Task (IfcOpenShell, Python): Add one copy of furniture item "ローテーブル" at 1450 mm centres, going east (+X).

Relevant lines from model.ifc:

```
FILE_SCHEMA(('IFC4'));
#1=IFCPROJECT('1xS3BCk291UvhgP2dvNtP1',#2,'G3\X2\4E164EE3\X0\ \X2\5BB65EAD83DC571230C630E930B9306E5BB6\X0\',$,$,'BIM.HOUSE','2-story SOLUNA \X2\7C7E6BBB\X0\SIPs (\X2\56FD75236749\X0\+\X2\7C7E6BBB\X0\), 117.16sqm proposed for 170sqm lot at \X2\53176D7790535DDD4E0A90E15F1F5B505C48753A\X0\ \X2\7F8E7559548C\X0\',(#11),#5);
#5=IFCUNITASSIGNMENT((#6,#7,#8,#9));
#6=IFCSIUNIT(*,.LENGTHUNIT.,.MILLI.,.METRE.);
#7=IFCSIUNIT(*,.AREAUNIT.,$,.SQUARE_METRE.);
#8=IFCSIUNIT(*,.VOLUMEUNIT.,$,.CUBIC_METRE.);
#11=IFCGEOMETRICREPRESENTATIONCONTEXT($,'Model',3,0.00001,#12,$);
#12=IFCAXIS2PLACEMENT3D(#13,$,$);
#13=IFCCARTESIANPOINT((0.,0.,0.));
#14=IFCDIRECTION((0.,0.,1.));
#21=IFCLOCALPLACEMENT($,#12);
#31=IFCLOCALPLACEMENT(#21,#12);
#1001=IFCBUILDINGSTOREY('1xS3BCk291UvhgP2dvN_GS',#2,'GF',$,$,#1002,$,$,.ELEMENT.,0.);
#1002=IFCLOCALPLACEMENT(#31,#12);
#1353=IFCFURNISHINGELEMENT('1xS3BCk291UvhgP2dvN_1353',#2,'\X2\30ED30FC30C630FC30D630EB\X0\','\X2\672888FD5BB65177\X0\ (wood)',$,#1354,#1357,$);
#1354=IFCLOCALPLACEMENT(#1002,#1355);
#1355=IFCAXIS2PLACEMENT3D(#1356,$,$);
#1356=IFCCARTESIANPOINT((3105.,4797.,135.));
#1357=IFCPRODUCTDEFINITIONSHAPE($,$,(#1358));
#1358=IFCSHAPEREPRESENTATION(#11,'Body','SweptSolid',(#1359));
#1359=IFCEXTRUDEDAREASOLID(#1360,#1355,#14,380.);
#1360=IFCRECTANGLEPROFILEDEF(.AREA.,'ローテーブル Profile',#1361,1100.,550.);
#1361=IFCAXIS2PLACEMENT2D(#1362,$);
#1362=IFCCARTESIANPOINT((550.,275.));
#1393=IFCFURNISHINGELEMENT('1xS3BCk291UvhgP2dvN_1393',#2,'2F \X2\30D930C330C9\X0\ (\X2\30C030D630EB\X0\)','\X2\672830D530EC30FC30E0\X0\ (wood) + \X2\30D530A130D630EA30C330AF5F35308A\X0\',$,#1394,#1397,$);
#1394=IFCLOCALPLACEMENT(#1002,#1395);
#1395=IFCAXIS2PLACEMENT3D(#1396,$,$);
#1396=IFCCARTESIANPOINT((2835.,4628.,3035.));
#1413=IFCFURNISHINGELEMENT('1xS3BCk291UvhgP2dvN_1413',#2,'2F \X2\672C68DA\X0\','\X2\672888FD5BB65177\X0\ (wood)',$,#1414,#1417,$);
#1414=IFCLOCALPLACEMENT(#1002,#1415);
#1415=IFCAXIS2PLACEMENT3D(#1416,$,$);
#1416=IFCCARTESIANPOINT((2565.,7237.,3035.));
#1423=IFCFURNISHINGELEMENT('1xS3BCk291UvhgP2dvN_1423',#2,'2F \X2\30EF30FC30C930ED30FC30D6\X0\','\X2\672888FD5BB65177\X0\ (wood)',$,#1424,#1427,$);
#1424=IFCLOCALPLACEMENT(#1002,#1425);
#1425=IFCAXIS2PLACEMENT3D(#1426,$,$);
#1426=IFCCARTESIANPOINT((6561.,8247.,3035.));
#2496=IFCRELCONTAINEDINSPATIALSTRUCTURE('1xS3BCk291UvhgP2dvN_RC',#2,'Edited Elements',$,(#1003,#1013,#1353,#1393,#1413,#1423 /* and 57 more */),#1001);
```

```python
import numpy as np
import ifcopenshell
import ifcopenshell.api.geometry
import ifcopenshell.api.root
import ifcopenshell.util.element
import ifcopenshell.util.placement
import ifcopenshell.util.unit

model = ifcopenshell.open("model.ifc")
unit_scale = ifcopenshell.util.unit.calculate_unit_scale(model)


def reuse_history(source, copy):
    """copy_class also copies each property set's owner history, people and application; keep the originals."""
    for rel in copy.IsDefinedBy:
        if rel.is_a("IfcRelDefinesByProperties") and (history := rel.RelatingPropertyDefinition.OwnerHistory):
            rel.RelatingPropertyDefinition.OwnerHistory = source.OwnerHistory
            ifcopenshell.util.element.remove_deep2(model, history)


source = model.by_id(1353)
base = ifcopenshell.util.placement.get_local_placement(source.ObjectPlacement)
step = np.array([1.0, 0.0, 0.0]) * 1.45 / unit_scale

for i in range(1, 2):
    copy = ifcopenshell.api.root.copy_class(model, product=source)
    copy.Representation = ifcopenshell.util.element.copy_deep(
        model, source.Representation, exclude=["IfcGeometricRepresentationContext", "IfcRepresentationMap"]
    )
    reuse_history(source, copy)
    matrix = base.copy()
    matrix[:3, 3] += i * step
    print("added at", matrix[:3, 3].round(3) + 0.0)
    ifcopenshell.api.geometry.edit_object_placement(model, product=copy, matrix=matrix, is_si=False)

model.write("model_updated.ifc")
```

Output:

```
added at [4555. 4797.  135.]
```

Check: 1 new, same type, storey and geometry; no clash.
